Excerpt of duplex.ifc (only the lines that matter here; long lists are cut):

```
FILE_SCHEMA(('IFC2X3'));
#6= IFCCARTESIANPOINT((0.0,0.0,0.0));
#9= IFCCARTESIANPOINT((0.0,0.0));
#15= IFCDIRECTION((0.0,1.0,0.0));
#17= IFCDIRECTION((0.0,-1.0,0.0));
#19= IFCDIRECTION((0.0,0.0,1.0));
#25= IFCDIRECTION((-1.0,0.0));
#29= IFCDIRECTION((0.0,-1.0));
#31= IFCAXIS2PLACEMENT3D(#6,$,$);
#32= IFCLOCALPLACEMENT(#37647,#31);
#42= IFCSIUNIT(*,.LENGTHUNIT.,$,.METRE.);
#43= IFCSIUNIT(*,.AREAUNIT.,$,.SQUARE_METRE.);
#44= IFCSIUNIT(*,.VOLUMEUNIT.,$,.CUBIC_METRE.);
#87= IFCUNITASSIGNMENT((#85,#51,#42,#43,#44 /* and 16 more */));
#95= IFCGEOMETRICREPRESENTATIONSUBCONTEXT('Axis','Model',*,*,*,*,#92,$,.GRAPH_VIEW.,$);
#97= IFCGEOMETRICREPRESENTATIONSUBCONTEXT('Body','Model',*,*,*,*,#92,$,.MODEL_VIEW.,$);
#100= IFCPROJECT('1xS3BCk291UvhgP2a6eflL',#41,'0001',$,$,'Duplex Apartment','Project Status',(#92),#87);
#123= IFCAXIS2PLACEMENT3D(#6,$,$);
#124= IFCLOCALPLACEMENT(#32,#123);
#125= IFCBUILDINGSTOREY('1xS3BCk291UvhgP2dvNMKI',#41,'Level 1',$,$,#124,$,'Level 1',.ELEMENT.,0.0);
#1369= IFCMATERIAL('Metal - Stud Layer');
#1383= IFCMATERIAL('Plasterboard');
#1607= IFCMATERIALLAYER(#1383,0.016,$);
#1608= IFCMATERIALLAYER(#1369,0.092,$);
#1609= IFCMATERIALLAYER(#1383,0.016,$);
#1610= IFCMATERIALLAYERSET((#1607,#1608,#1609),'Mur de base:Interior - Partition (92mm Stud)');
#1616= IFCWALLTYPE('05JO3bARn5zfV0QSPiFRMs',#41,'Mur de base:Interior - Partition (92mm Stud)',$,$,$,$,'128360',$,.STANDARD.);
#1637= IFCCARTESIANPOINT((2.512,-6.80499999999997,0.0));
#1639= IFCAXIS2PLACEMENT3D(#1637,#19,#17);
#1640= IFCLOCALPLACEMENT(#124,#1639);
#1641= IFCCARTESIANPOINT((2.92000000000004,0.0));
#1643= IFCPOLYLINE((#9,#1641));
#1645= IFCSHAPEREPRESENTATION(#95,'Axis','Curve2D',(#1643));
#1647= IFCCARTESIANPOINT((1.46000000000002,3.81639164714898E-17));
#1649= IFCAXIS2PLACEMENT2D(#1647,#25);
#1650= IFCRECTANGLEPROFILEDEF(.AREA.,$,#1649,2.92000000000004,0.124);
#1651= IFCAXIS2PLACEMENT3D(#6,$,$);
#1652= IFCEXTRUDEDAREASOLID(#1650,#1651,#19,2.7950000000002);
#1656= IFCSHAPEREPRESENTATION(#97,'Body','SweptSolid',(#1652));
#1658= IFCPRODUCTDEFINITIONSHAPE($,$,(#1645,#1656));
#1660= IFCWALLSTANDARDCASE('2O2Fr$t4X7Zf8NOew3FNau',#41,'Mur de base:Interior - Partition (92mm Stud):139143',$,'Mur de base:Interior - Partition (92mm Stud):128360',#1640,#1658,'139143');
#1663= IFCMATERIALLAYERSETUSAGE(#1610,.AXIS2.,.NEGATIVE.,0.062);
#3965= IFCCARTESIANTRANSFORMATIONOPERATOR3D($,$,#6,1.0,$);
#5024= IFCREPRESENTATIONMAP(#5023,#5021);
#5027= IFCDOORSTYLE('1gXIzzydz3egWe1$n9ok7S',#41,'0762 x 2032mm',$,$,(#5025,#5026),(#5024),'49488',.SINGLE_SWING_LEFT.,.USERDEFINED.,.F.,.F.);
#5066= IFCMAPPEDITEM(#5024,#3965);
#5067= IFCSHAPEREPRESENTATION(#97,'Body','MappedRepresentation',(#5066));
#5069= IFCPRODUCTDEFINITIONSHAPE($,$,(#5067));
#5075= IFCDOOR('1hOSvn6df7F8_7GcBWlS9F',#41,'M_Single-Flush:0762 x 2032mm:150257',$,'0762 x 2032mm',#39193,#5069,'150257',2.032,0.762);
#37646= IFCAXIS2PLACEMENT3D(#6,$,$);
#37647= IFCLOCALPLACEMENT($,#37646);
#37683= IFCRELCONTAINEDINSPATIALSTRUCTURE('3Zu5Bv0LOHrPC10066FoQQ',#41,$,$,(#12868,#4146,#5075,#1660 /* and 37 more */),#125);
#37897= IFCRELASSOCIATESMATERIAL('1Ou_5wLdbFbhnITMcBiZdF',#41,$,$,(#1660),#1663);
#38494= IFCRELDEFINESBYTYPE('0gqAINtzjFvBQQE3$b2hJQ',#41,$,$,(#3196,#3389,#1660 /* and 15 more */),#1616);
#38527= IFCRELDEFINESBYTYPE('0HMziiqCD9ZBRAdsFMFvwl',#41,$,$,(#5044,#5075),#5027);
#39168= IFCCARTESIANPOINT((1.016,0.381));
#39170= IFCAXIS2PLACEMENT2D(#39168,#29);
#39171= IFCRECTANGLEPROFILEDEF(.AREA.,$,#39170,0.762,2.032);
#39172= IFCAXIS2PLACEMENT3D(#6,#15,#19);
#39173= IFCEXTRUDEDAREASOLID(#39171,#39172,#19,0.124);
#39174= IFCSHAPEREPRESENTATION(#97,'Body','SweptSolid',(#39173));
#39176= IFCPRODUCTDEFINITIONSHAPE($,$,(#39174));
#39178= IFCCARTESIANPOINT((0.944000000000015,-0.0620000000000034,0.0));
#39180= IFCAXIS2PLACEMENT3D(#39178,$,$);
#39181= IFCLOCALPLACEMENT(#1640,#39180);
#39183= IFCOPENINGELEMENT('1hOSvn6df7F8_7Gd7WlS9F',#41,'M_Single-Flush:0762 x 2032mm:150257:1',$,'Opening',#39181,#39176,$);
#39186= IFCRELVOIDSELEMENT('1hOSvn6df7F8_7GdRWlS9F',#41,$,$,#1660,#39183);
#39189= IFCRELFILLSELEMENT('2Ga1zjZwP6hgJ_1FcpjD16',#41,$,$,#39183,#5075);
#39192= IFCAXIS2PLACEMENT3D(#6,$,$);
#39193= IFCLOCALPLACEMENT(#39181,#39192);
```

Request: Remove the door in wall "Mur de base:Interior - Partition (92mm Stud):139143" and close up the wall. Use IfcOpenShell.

```python
import ifcopenshell
import ifcopenshell.api.feature
import ifcopenshell.api.root
import ifcopenshell.geom
import ifcopenshell.util.shape

model = ifcopenshell.open("duplex.ifc")
settings = ifcopenshell.geom.settings()


def volume(element):
    """Net volume in cubic metres, openings subtracted."""
    shape = ifcopenshell.geom.create_shape(settings, element)
    return ifcopenshell.util.shape.get_volume(shape.geometry)


door = model.by_guid("1hOSvn6df7F8_7GcBWlS9F")
opening = door.FillsVoids[0].RelatingOpeningElement
wall = opening.VoidsElements[0].RelatingBuildingElement
before = volume(wall)

ifcopenshell.api.root.remove_product(model, product=door)
ifcopenshell.api.feature.remove_feature(model, feature=opening)

after = volume(wall)

print(f"wall volume {before:.3f} -> {after:.3f} m3")

model.write("duplex_rev.ifc")
```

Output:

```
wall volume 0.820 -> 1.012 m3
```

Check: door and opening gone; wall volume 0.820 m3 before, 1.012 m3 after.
